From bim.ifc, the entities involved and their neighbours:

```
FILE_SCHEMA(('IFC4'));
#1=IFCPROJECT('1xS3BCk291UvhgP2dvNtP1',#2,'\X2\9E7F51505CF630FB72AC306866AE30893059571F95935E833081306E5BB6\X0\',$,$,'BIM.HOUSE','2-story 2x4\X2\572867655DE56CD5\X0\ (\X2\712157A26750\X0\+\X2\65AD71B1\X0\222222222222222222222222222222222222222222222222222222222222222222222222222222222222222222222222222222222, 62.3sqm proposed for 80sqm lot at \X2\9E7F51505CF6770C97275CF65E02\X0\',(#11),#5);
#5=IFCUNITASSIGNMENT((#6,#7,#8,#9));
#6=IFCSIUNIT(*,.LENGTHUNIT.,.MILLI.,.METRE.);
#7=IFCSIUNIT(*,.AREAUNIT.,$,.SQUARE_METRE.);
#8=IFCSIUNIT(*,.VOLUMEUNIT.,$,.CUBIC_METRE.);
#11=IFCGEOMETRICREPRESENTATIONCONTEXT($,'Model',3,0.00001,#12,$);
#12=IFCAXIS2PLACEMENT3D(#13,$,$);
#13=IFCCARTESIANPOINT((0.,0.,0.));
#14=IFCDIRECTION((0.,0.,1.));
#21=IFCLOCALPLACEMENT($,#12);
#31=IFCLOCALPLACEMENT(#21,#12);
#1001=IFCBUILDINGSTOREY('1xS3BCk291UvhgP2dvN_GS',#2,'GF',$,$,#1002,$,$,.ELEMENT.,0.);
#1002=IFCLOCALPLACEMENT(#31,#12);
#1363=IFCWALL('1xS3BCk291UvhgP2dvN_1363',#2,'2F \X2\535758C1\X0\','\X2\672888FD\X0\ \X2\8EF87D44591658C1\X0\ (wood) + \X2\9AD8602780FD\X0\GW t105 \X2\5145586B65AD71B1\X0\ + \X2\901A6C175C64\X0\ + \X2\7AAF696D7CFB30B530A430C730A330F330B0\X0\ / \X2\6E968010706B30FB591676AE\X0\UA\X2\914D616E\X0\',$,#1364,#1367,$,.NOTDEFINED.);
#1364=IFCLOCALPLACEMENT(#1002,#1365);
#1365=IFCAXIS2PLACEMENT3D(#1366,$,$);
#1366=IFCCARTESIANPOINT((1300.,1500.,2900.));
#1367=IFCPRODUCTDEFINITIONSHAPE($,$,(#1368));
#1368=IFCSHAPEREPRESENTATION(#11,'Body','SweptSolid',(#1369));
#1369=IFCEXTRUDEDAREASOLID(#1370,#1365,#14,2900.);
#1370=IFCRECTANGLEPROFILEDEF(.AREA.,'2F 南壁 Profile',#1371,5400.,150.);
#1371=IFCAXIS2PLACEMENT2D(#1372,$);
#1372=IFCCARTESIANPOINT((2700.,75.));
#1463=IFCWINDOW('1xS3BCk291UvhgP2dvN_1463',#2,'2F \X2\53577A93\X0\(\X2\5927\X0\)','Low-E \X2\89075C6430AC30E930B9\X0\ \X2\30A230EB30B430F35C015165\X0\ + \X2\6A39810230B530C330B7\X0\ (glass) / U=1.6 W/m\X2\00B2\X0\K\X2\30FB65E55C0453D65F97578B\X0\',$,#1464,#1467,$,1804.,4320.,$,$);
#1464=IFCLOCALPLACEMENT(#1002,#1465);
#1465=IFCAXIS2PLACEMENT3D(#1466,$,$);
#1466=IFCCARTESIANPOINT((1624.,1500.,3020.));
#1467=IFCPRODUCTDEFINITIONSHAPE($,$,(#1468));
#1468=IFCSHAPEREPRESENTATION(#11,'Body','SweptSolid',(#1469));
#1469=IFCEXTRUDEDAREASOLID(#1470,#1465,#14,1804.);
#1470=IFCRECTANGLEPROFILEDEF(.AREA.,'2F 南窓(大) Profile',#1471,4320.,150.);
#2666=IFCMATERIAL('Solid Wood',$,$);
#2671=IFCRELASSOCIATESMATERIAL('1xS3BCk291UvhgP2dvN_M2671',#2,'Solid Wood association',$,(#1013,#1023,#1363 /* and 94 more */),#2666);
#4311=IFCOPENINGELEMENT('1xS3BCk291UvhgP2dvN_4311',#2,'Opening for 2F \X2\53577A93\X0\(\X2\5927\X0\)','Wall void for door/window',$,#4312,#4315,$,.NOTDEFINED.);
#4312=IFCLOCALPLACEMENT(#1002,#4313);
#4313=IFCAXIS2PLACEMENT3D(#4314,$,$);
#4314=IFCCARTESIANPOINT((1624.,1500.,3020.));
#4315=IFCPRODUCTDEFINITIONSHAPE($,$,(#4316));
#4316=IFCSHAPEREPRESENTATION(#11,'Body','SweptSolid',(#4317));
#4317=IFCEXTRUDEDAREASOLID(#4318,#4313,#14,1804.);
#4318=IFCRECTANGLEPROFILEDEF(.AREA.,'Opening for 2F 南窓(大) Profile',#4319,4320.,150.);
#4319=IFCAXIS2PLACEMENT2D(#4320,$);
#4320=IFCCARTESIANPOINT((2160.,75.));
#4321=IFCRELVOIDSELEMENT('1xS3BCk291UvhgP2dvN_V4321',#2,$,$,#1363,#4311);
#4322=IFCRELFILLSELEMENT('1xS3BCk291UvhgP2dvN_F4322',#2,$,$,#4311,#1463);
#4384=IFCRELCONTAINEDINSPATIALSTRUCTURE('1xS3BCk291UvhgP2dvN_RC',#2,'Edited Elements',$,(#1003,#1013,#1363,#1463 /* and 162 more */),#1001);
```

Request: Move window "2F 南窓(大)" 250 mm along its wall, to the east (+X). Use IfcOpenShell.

```python
import ifcopenshell
import ifcopenshell.api.geometry
import ifcopenshell.util.placement
import ifcopenshell.util.unit

model = ifcopenshell.open("bim.ifc")
unit_scale = ifcopenshell.util.unit.calculate_unit_scale(model)

window = model.by_guid("1xS3BCk291UvhgP2dvN_1463")
opening = window.FillsVoids[0].RelatingOpeningElement
wall = opening.VoidsElements[0].RelatingBuildingElement

wall_matrix = ifcopenshell.util.placement.get_local_placement(wall.ObjectPlacement)
shift = wall_matrix[:3, 0] * 0.25 / unit_scale
before = ifcopenshell.util.placement.get_local_placement(window.ObjectPlacement)[:3, 3].copy()

# The window is not placed relative to its opening, so move both.
for product in (opening, window):
    matrix = ifcopenshell.util.placement.get_local_placement(product.ObjectPlacement)
    matrix[:3, 3] += shift
    ifcopenshell.api.geometry.edit_object_placement(model, product=product, matrix=matrix, is_si=False)

after = ifcopenshell.util.placement.get_local_placement(window.ObjectPlacement)[:3, 3]
print("window moved by", (after - before).round(3) + 0.0)

model.write("bim_edited.ifc")
```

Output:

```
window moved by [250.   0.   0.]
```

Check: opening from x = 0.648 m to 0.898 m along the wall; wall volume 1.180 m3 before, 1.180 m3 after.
